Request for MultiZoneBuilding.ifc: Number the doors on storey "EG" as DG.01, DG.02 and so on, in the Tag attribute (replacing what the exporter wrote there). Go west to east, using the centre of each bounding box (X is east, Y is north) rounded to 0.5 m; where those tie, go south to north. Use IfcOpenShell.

First a look at what the model holds.

```python
import ifcopenshell
import ifcopenshell.util.element
import ifcopenshell.util.placement

model = ifcopenshell.open("MultiZoneBuilding.ifc")
print(model.schema)
storey = next(s for s in model.by_type("IfcBuildingStorey") if s.Name == "EG")
doors = [e for e in ifcopenshell.util.element.get_decomposition(storey) if e.is_a("IfcDoor")]
for e in sorted(doors, key=lambda e: e.id()):
    origin = ifcopenshell.util.placement.get_local_placement(e.ObjectPlacement)[:3, 3]
    print(e.id(), e.Tag, e.Name, origin.round(2) + 0.0, sep=" | ")
```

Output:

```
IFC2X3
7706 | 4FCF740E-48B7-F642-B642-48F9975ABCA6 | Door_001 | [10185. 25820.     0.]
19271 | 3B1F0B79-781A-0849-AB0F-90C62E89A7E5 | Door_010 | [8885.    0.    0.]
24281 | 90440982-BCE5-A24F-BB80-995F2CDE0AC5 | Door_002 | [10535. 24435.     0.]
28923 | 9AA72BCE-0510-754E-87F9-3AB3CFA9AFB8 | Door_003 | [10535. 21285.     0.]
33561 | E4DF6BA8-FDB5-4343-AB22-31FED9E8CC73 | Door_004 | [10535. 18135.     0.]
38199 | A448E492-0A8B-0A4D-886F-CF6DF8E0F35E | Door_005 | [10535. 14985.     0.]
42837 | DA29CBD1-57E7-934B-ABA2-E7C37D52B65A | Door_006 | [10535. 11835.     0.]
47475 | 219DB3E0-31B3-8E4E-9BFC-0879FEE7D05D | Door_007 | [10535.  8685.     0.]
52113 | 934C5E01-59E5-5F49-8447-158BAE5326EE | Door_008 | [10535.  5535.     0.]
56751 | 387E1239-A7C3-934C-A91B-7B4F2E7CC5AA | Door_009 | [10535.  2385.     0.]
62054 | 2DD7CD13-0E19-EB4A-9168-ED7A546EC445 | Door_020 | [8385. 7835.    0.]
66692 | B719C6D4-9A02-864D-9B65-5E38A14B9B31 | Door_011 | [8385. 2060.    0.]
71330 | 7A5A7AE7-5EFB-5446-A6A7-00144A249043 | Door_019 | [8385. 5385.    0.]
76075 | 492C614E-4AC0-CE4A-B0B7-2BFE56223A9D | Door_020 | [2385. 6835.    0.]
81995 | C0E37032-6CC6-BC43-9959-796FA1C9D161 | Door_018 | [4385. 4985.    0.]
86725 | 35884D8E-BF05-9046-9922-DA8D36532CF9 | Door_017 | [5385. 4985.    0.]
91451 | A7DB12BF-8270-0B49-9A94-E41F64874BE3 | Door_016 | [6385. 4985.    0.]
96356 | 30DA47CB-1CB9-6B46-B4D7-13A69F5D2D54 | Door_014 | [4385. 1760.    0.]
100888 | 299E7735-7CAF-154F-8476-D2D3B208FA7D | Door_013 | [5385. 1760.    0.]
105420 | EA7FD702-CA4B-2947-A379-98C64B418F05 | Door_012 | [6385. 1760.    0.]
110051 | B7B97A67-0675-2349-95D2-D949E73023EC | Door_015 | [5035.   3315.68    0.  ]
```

```python
import ifcopenshell
import ifcopenshell.geom
import ifcopenshell.util.element
import ifcopenshell.util.shape

model = ifcopenshell.open("MultiZoneBuilding.ifc")
settings = ifcopenshell.geom.settings()
settings.set("use-world-coords", True)


def centre(element):
    shape = ifcopenshell.geom.create_shape(settings, element)
    return ifcopenshell.util.shape.get_bbox_centroid(shape.geometry)


storey = next(s for s in model.by_type("IfcBuildingStorey") if s.Name == "EG")
doors = [e for e in ifcopenshell.util.element.get_decomposition(storey) if e.is_a("IfcDoor")]

# Insertion points can sit at a corner or the storey origin, so sort by the geometry (in metres).
centres = {e: centre(e) for e in doors}
doors.sort(key=lambda e: (round(centres[e][0] / 0.5), centres[e][1]))

for i, e in enumerate(doors, start=1):
    number = f"DG.{i:02d}"
    e.Tag = number
    print(e.id(), number)

model.write("MultiZoneBuilding_v2.ifc")
```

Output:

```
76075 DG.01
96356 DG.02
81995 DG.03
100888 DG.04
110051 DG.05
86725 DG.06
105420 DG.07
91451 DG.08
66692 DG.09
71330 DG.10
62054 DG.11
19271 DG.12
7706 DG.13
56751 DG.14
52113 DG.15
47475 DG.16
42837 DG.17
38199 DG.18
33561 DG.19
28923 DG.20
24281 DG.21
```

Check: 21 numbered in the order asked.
